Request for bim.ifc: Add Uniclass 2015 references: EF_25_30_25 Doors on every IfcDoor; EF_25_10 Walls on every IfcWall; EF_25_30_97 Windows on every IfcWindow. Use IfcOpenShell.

First a look at what the model holds.

```python
import ifcopenshell

model = ifcopenshell.open("bim.ifc")
print(model.schema)
print("classifications:", [c.Name for c in model.by_type("IfcClassification")])
for ifc_class in ("IfcDoor", "IfcRoof", "IfcStair", "IfcWall", "IfcWindow"):
    print(ifc_class, len(model.by_type(ifc_class)))
```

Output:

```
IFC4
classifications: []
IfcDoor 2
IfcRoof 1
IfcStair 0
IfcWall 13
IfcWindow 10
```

```python
import ifcopenshell
import ifcopenshell.api.classification

model = ifcopenshell.open("bim.ifc")

system = ifcopenshell.api.classification.add_classification(model, classification="Uniclass 2015")

codes = {
    "IfcDoor": ("EF_25_30_25", "Doors"),
    "IfcWall": ("EF_25_10", "Walls"),
    "IfcWindow": ("EF_25_30_97", "Windows"),
}
for ifc_class, (code, name) in codes.items():
    products = model.by_type(ifc_class)
    ifcopenshell.api.classification.add_reference(
        model, products=products, classification=system, identification=code, name=name
    )
    print(code, len(products))

model.write("bim-out.ifc")
```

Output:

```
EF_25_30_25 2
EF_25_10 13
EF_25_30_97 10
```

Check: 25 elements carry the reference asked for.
